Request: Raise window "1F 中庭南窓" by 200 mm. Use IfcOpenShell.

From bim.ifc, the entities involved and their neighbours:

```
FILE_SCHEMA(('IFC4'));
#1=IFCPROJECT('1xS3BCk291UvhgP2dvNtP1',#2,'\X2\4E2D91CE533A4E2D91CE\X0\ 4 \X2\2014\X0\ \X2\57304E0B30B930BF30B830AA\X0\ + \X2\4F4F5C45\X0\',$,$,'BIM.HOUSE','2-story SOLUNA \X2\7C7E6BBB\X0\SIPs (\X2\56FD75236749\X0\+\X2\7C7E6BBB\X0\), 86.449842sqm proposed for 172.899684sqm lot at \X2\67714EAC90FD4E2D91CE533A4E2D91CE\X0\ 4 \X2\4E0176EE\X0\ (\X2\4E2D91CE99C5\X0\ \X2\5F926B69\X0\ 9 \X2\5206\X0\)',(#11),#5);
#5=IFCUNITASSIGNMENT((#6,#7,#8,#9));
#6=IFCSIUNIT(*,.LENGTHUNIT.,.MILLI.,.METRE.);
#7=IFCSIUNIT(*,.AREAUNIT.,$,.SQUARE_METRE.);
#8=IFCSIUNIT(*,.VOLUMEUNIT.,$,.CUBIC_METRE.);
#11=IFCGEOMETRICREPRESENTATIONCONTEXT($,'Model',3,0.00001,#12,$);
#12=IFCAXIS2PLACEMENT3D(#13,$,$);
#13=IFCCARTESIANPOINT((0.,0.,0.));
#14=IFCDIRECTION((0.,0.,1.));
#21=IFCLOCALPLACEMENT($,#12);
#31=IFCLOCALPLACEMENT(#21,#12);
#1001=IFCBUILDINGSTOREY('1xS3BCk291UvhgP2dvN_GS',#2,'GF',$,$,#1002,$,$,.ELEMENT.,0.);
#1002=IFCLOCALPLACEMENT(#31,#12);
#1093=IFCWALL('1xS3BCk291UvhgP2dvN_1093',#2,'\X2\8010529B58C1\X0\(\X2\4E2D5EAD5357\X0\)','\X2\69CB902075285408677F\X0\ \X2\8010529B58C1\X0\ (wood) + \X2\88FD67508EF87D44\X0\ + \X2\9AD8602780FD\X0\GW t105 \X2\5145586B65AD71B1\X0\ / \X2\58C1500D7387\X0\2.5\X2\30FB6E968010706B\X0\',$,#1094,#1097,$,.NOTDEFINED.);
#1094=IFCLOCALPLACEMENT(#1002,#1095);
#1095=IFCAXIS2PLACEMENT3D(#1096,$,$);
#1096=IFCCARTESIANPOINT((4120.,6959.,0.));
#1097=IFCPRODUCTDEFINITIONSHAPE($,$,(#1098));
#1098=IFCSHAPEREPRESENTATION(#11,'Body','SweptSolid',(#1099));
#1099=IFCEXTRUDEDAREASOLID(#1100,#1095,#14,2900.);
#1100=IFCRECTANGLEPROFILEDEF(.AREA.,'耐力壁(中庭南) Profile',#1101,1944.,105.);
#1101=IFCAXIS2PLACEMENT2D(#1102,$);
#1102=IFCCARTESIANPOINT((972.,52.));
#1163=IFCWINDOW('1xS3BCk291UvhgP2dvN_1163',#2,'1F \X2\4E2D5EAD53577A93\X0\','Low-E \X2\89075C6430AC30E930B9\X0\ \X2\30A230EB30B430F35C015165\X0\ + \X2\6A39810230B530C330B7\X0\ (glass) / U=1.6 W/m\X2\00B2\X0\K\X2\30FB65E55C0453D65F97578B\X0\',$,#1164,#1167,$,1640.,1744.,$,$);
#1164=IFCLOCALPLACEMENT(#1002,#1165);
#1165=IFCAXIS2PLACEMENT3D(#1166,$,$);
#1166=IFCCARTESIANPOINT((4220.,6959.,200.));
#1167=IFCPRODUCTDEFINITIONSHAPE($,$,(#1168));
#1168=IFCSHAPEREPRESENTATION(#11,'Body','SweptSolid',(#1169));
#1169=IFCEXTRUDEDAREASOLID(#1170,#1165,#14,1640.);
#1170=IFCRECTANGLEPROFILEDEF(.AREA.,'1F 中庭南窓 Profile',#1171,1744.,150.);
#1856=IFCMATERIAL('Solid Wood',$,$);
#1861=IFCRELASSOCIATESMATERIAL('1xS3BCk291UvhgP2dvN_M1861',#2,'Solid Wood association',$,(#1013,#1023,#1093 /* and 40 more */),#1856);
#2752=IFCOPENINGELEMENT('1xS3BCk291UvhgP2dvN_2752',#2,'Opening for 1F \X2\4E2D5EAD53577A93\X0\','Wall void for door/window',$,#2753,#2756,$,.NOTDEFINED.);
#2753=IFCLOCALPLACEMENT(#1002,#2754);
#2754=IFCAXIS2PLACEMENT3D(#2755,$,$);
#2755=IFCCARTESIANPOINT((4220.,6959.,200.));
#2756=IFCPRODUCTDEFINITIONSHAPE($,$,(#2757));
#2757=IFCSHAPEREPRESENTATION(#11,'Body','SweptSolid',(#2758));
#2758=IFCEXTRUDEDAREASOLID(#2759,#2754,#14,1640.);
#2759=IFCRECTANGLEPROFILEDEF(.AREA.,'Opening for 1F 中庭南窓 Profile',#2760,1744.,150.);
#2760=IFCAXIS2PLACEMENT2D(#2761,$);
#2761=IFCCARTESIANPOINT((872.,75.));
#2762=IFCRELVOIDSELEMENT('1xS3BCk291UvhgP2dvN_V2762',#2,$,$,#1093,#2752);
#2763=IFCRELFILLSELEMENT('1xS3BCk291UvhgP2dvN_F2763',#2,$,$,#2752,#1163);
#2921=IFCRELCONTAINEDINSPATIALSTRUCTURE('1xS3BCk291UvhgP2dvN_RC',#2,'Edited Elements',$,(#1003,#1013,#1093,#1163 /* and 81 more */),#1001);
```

```python
import numpy as np
import ifcopenshell
import ifcopenshell.api.geometry
import ifcopenshell.util.placement
import ifcopenshell.util.unit

model = ifcopenshell.open("bim.ifc")
unit_scale = ifcopenshell.util.unit.calculate_unit_scale(model)

window = model.by_guid("1xS3BCk291UvhgP2dvN_1163")
opening = window.FillsVoids[0].RelatingOpeningElement
dz = 0.2 / unit_scale

shift = np.array([0.0, 0.0, dz])
# The window is not placed relative to its opening, so move both.
for product in (opening, window):
    matrix = ifcopenshell.util.placement.get_local_placement(product.ObjectPlacement)
    matrix[:3, 3] += shift
    ifcopenshell.api.geometry.edit_object_placement(model, product=product, matrix=matrix, is_si=False)

print(f"moved by {dz * unit_scale:+.3f} m")

model.write("bim_edited.ifc")
```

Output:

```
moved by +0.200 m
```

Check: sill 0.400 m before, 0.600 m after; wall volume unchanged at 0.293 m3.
